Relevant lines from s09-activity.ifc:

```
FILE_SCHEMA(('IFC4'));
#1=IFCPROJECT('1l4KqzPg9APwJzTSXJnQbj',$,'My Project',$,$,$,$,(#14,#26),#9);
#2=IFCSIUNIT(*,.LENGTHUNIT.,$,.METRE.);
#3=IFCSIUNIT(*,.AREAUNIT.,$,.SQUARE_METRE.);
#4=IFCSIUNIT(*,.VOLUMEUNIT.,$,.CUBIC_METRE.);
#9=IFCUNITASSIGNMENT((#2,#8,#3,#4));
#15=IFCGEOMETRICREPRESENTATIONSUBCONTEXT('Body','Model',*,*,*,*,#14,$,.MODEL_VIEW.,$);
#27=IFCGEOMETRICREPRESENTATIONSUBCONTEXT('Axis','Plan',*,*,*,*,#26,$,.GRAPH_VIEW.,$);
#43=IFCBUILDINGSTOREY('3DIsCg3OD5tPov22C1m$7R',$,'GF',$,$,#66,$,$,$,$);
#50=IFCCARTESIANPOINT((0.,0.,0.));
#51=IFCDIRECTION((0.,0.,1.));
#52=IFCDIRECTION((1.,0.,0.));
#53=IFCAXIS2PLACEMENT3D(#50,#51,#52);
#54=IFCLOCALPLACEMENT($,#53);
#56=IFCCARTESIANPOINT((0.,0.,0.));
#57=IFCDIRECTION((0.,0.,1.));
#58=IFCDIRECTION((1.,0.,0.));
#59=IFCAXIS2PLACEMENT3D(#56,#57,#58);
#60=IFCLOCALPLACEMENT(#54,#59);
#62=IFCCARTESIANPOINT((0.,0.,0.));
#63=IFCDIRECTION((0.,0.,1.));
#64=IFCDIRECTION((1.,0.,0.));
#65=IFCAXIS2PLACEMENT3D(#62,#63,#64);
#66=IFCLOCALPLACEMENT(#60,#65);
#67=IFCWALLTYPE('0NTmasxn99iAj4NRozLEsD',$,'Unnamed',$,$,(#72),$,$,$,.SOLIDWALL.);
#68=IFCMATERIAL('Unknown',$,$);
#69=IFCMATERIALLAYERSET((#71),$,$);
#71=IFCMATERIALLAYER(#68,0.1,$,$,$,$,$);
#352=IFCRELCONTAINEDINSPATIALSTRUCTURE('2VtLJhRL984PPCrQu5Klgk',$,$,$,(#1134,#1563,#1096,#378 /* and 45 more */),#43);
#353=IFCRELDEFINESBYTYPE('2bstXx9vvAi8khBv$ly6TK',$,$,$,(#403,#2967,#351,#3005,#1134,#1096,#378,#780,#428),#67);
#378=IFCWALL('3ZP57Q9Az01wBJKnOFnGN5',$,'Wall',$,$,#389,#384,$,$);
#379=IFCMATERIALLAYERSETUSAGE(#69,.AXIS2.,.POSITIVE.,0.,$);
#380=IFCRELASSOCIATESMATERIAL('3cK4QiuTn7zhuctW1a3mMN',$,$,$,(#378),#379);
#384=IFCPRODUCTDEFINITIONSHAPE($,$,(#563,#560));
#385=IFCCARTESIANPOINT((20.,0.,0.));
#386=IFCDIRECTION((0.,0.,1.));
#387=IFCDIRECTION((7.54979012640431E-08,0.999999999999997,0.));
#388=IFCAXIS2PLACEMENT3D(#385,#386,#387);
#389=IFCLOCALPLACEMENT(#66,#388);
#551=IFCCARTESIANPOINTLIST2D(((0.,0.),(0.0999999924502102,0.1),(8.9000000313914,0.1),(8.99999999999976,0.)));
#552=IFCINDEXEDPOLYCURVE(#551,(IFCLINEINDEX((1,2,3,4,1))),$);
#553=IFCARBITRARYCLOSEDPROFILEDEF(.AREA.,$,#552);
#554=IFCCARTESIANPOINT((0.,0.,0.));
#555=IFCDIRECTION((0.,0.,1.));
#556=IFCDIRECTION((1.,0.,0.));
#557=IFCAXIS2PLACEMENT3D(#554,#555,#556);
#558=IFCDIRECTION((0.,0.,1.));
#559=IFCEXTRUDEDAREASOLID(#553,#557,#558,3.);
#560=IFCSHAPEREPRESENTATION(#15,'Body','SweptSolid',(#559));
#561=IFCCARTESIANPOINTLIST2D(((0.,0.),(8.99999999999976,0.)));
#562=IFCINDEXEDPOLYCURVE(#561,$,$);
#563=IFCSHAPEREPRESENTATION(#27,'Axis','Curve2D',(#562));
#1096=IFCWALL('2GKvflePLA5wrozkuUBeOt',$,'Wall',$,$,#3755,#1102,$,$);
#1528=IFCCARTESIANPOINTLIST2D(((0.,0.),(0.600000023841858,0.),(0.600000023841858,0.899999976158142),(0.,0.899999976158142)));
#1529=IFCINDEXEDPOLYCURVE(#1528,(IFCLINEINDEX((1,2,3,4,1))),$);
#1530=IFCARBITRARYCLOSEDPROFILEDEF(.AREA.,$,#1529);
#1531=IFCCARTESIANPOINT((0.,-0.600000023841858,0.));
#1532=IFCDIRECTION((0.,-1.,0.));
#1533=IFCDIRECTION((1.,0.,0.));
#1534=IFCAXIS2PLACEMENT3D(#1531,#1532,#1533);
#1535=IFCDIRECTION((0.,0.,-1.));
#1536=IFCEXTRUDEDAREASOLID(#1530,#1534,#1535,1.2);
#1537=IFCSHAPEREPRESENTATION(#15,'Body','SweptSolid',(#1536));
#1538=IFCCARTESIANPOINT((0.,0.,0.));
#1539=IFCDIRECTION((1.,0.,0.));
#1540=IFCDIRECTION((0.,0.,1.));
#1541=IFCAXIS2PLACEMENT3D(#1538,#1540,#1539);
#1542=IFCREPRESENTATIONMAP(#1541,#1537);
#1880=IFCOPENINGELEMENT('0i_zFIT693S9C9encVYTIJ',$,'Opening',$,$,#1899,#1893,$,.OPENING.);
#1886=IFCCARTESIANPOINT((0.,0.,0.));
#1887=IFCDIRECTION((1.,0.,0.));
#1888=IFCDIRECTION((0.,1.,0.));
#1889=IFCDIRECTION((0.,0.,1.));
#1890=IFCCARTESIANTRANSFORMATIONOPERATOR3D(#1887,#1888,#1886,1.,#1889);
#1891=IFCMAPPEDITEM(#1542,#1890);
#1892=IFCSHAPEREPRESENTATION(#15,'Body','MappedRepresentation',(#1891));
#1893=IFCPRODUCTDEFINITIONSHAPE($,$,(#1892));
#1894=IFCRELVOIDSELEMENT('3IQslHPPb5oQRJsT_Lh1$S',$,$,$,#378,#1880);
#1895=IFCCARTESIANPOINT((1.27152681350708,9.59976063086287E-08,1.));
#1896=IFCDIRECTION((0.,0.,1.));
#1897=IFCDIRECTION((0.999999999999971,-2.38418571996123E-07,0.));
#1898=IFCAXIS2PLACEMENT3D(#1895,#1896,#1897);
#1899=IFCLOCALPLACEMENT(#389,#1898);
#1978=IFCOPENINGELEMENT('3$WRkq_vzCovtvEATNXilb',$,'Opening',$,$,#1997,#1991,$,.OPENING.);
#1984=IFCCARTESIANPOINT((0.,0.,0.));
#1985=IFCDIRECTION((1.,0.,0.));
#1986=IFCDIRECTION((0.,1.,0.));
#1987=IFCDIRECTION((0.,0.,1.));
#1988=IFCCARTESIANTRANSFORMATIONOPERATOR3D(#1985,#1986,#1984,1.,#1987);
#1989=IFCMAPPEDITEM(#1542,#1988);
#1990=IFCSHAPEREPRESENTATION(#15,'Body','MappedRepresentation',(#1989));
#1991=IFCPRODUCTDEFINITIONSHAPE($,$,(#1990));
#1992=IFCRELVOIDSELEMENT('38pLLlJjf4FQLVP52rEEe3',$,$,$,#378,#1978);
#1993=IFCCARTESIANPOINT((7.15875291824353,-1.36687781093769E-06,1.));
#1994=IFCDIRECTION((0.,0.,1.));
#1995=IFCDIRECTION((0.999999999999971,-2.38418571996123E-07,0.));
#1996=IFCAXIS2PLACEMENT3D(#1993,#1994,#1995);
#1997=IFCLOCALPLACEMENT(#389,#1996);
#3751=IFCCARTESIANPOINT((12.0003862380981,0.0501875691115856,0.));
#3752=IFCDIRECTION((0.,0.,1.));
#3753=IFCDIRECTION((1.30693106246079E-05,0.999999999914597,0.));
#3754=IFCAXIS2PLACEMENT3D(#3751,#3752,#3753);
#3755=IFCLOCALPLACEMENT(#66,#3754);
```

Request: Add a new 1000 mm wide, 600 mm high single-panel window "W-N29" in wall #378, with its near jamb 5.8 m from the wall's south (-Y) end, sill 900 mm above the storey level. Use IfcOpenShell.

```python
import numpy as np
import ifcopenshell
import ifcopenshell.api.feature
import ifcopenshell.api.geometry
import ifcopenshell.api.root
import ifcopenshell.api.spatial
import ifcopenshell.geom
import ifcopenshell.util.element
import ifcopenshell.util.placement
import ifcopenshell.util.representation
import ifcopenshell.util.shape
import ifcopenshell.util.unit

model = ifcopenshell.open("s09-activity.ifc")
unit_scale = ifcopenshell.util.unit.calculate_unit_scale(model)
settings = ifcopenshell.geom.settings()


def volume(element):
    """Net volume in cubic metres, openings subtracted."""
    shape = ifcopenshell.geom.create_shape(settings, element)
    return ifcopenshell.util.shape.get_volume(shape.geometry)


wall = model.by_guid("3ZP57Q9Az01wBJKnOFnGN5")
storey = ifcopenshell.util.element.get_container(wall, ifc_class="IfcBuildingStorey")
context = ifcopenshell.util.representation.get_context(model, "Model", "Body", "MODEL_VIEW")
before = volume(wall)

width, height, from_end, sill = 1, 0.6, 5.8, 0.9  # metres

# The wall runs along its own X axis, and the end named is its -X end.
wall_shape = ifcopenshell.geom.create_shape(settings, wall)
x, y, z = ifcopenshell.util.shape.get_vertices(wall_shape.geometry).T
start = x.min() + from_end
face, thickness = float(y.min()), float(y.max() - y.min())
wall_matrix = ifcopenshell.util.placement.get_local_placement(wall.ObjectPlacement)
level = ifcopenshell.util.placement.get_local_placement(storey.ObjectPlacement)[2, 3]


def in_wall(x, y):
    """Placement at x, y metres in the wall's axes, at sill height."""
    matrix = wall_matrix.copy()
    matrix[:, 3] = wall_matrix @ np.array([x / unit_scale, y / unit_scale, 0.0, 1.0])
    matrix[2, 3] = level + sill / unit_scale
    return matrix


# Opening: a box that overshoots both wall faces by 50 mm.
opening = ifcopenshell.api.root.create_entity(model, ifc_class="IfcOpeningElement", predefined_type="OPENING")
box = ifcopenshell.api.geometry.add_wall_representation(
    model, context=context, length=width, height=height, thickness=thickness + 0.1
)
ifcopenshell.api.geometry.assign_representation(model, product=opening, representation=box)
ifcopenshell.api.geometry.edit_object_placement(model, product=opening, matrix=in_wall(start, face - 0.05), is_si=False)
ifcopenshell.api.feature.add_feature(model, feature=opening, element=wall)

window = ifcopenshell.api.root.create_entity(model, ifc_class="IfcWindow", name="W-N29", predefined_type="WINDOW")
window.OverallWidth, window.OverallHeight = width / unit_scale, height / unit_scale
window.PartitioningType = "SINGLE_PANEL"
body = ifcopenshell.api.geometry.add_window_representation(
    model,
    context=context,
    overall_width=window.OverallWidth,
    overall_height=window.OverallHeight,
    partition_type="SINGLE_PANEL",
)
ifcopenshell.api.geometry.assign_representation(model, product=window, representation=body)
ifcopenshell.api.spatial.assign_container(model, products=[window], relating_structure=storey)
ifcopenshell.api.feature.add_filling(model, opening=opening, element=window)

# Centre the window in the wall's thickness.
ifcopenshell.api.geometry.edit_object_placement(model, product=window, matrix=in_wall(start, face), is_si=False)
window_shape = ifcopenshell.geom.create_shape(settings, window)
depth = ifcopenshell.util.shape.get_vertices(window_shape.geometry)[:, 1]
offset = face + thickness / 2 - (depth.min() + depth.max()) / 2
ifcopenshell.api.geometry.edit_object_placement(model, product=window, matrix=in_wall(start, offset), is_si=False)

after = volume(wall)

print(f"wall volume {before:.3f} -> {after:.3f} m3")

model.write("s09-activity_v2.ifc")
```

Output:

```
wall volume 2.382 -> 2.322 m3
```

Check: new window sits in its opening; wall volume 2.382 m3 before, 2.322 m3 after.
